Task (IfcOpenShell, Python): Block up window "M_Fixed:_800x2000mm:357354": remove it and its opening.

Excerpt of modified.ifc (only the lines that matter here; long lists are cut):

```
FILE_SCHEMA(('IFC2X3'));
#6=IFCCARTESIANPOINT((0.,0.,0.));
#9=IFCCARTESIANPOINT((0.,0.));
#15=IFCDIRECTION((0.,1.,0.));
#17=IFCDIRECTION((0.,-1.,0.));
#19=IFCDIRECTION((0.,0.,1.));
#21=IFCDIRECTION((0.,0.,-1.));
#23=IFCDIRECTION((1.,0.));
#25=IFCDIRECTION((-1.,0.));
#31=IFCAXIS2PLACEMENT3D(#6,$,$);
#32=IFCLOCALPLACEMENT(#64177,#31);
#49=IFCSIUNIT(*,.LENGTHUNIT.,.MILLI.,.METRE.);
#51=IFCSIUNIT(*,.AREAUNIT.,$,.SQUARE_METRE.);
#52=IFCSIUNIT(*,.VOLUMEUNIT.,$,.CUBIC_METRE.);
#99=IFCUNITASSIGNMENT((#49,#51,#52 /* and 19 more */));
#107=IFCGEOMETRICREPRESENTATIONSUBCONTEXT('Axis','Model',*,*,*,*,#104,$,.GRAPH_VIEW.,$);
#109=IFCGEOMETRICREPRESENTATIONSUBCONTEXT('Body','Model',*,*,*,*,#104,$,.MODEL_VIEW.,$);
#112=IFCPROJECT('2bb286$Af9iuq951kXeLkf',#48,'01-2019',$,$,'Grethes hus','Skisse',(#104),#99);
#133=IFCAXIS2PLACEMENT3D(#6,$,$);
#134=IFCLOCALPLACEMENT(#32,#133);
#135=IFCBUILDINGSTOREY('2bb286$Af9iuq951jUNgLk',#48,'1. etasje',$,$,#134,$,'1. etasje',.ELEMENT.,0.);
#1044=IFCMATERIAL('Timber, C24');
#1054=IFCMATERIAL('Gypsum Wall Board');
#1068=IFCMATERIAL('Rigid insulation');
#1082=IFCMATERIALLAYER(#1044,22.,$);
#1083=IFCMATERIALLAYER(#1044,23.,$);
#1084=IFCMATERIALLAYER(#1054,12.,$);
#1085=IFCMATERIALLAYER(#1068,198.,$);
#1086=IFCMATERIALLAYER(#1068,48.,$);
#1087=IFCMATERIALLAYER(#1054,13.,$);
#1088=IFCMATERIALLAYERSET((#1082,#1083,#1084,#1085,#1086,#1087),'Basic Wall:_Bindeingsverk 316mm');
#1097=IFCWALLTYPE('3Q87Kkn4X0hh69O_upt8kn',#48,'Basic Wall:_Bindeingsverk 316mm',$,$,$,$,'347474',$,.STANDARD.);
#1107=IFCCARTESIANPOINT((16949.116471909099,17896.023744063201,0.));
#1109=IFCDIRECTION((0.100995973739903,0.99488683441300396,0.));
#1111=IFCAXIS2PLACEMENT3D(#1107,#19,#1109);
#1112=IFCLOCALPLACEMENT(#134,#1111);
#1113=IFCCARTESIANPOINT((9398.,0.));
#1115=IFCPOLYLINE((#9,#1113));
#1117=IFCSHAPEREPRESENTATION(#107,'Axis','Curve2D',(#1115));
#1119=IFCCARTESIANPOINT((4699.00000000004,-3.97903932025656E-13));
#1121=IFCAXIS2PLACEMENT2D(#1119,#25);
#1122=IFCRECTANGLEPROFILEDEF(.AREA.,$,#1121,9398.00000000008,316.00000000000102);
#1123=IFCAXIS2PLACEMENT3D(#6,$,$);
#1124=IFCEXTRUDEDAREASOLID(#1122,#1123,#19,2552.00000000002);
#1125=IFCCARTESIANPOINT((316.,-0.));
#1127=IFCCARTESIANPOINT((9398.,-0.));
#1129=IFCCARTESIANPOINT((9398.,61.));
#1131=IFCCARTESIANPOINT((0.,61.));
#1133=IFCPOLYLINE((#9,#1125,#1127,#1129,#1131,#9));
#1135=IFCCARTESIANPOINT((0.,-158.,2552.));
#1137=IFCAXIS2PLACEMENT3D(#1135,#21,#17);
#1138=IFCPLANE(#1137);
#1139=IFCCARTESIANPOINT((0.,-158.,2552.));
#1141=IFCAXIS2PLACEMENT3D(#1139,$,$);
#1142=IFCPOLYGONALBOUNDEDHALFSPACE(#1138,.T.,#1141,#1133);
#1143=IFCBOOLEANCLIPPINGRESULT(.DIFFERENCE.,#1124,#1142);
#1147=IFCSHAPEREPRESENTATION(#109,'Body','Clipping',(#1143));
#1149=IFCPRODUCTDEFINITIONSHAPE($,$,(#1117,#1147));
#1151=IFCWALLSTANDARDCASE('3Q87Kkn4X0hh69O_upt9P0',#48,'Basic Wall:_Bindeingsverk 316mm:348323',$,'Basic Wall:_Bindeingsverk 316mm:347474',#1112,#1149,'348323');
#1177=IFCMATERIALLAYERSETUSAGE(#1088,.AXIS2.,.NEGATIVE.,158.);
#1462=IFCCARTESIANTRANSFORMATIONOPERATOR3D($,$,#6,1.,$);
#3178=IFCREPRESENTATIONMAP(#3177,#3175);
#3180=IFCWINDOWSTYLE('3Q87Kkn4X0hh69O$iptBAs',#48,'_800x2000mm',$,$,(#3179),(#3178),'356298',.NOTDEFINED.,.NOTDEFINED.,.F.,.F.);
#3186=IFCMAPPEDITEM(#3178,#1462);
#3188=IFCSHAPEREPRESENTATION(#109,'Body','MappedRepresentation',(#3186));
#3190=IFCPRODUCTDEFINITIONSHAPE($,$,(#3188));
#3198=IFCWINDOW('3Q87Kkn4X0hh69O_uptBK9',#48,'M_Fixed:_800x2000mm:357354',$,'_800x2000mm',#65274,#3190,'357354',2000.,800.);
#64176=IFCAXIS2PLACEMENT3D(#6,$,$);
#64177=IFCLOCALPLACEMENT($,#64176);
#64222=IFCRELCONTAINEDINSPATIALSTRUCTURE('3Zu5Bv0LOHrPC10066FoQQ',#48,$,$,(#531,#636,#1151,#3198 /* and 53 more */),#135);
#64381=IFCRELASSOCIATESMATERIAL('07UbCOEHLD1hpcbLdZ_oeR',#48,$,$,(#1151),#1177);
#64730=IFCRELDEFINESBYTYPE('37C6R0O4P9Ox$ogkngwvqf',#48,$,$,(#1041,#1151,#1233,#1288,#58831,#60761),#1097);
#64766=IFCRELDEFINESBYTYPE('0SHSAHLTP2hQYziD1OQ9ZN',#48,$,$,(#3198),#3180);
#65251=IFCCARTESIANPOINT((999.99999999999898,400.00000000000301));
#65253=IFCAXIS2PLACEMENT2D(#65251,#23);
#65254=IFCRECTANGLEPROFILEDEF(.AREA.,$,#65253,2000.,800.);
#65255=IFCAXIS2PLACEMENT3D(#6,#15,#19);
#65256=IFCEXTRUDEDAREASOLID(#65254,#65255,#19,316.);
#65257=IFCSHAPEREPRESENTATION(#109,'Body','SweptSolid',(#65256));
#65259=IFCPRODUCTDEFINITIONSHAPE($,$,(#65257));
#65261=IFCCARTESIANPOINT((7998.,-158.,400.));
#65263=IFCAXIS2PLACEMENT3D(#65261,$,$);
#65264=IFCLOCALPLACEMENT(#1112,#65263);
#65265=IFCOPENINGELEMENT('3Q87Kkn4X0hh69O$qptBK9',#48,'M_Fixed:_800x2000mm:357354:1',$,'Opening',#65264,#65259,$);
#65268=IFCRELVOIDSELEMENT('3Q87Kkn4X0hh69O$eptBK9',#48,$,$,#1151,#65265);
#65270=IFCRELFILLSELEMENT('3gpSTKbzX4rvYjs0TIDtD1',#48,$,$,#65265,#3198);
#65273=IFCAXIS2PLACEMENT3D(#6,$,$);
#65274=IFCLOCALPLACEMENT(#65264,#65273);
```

```python
import ifcopenshell
import ifcopenshell.api.feature
import ifcopenshell.api.root
import ifcopenshell.geom
import ifcopenshell.util.shape

model = ifcopenshell.open("modified.ifc")
settings = ifcopenshell.geom.settings()


def volume(element):
    """Net volume in cubic metres, openings subtracted."""
    shape = ifcopenshell.geom.create_shape(settings, element)
    return ifcopenshell.util.shape.get_volume(shape.geometry)


window = model.by_id(3198)
opening = window.FillsVoids[0].RelatingOpeningElement
wall = opening.VoidsElements[0].RelatingBuildingElement
before = volume(wall)

ifcopenshell.api.root.remove_product(model, product=window)
ifcopenshell.api.feature.remove_feature(model, feature=opening)

after = volume(wall)

print(f"wall volume {before:.3f} -> {after:.3f} m3")

model.write("modified_rev.ifc")
```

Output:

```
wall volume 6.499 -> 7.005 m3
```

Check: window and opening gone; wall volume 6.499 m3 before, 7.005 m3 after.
